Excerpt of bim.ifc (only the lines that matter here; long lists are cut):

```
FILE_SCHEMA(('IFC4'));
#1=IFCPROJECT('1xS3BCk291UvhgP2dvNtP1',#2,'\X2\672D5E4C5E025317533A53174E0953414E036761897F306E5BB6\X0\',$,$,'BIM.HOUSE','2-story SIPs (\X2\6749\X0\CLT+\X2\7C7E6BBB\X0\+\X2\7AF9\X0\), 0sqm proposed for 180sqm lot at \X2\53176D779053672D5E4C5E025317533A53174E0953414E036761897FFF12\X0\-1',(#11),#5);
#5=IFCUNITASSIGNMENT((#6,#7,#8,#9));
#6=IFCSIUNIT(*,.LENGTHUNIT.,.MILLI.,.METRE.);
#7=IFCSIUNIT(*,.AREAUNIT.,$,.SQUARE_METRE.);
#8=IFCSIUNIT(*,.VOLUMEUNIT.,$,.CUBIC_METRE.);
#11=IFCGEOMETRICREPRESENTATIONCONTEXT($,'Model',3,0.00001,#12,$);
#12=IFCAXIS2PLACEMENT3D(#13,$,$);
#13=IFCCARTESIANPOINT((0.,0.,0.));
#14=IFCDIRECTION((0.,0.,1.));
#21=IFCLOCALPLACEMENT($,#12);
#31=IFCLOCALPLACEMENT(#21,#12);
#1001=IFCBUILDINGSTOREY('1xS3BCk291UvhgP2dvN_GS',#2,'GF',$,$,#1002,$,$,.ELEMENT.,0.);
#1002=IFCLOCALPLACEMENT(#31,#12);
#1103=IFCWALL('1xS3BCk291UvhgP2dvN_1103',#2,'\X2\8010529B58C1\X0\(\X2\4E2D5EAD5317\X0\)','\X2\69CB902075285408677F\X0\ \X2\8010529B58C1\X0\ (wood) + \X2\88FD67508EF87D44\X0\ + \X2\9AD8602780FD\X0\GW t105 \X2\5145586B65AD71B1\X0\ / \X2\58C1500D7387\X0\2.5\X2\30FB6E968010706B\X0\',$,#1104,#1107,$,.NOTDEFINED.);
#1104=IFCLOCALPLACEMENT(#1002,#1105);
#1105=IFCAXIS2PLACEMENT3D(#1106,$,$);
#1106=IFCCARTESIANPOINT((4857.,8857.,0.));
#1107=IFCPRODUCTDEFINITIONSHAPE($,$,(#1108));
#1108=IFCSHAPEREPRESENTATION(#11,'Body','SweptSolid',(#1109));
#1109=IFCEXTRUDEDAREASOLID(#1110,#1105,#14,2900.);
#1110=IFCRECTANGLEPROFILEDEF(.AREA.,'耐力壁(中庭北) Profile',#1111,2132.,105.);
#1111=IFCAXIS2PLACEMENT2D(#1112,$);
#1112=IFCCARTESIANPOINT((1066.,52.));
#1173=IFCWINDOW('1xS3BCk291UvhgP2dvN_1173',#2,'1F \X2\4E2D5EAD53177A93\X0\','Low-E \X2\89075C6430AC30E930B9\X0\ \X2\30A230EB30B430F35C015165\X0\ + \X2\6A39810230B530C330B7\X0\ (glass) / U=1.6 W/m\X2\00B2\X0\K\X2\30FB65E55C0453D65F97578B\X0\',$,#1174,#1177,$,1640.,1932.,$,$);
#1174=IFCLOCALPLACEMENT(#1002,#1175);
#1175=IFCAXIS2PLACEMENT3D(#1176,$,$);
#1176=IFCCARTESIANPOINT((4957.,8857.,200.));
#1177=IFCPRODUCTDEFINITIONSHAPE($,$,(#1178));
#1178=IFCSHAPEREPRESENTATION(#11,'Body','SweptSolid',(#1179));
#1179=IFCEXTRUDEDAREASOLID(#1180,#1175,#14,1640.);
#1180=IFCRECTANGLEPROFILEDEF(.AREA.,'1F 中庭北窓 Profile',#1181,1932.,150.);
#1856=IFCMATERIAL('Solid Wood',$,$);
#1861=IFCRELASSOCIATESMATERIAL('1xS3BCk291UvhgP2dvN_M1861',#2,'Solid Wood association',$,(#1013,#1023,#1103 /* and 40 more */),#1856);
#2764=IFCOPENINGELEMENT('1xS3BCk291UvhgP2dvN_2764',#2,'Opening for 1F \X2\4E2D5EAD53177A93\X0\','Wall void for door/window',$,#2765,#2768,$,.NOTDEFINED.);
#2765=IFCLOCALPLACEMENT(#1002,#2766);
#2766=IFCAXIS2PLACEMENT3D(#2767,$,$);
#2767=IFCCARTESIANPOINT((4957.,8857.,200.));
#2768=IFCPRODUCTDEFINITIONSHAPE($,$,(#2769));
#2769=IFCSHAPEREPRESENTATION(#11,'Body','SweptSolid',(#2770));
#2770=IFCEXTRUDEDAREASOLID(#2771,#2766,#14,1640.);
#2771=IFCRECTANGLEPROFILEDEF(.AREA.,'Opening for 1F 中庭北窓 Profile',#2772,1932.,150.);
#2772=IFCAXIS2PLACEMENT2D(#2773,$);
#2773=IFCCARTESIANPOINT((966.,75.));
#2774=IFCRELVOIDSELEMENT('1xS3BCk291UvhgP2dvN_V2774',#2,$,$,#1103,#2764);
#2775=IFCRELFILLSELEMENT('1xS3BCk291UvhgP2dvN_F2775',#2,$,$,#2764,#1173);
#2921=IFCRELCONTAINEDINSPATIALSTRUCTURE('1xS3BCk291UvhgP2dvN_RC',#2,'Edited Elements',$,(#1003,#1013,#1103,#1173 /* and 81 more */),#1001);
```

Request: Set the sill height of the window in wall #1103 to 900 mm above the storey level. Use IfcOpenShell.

```python
import numpy as np
import ifcopenshell
import ifcopenshell.api.geometry
import ifcopenshell.geom
import ifcopenshell.util.element
import ifcopenshell.util.placement
import ifcopenshell.util.shape
import ifcopenshell.util.unit

model = ifcopenshell.open("bim.ifc")
unit_scale = ifcopenshell.util.unit.calculate_unit_scale(model)

window = model.by_guid("1xS3BCk291UvhgP2dvN_1173")
opening = window.FillsVoids[0].RelatingOpeningElement
storey = ifcopenshell.util.element.get_container(window, ifc_class="IfcBuildingStorey")
level = ifcopenshell.util.placement.get_local_placement(storey.ObjectPlacement)[2, 3]

# The opening's origin need not be at the sill, so measure its lowest point.
shape = ifcopenshell.geom.create_shape(ifcopenshell.geom.settings(), opening)
bottom = ifcopenshell.util.shape.get_shape_bottom_elevation(shape, shape.geometry) / unit_scale
dz = level + 900.0 - bottom

shift = np.array([0.0, 0.0, dz])
# The window is not placed relative to its opening, so move both.
for product in (opening, window):
    matrix = ifcopenshell.util.placement.get_local_placement(product.ObjectPlacement)
    matrix[:3, 3] += shift
    ifcopenshell.api.geometry.edit_object_placement(model, product=product, matrix=matrix, is_si=False)

print(f"moved by {dz * unit_scale:+.3f} m")

model.write("bim_updated.ifc")
```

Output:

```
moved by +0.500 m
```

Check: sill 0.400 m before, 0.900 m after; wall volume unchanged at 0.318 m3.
